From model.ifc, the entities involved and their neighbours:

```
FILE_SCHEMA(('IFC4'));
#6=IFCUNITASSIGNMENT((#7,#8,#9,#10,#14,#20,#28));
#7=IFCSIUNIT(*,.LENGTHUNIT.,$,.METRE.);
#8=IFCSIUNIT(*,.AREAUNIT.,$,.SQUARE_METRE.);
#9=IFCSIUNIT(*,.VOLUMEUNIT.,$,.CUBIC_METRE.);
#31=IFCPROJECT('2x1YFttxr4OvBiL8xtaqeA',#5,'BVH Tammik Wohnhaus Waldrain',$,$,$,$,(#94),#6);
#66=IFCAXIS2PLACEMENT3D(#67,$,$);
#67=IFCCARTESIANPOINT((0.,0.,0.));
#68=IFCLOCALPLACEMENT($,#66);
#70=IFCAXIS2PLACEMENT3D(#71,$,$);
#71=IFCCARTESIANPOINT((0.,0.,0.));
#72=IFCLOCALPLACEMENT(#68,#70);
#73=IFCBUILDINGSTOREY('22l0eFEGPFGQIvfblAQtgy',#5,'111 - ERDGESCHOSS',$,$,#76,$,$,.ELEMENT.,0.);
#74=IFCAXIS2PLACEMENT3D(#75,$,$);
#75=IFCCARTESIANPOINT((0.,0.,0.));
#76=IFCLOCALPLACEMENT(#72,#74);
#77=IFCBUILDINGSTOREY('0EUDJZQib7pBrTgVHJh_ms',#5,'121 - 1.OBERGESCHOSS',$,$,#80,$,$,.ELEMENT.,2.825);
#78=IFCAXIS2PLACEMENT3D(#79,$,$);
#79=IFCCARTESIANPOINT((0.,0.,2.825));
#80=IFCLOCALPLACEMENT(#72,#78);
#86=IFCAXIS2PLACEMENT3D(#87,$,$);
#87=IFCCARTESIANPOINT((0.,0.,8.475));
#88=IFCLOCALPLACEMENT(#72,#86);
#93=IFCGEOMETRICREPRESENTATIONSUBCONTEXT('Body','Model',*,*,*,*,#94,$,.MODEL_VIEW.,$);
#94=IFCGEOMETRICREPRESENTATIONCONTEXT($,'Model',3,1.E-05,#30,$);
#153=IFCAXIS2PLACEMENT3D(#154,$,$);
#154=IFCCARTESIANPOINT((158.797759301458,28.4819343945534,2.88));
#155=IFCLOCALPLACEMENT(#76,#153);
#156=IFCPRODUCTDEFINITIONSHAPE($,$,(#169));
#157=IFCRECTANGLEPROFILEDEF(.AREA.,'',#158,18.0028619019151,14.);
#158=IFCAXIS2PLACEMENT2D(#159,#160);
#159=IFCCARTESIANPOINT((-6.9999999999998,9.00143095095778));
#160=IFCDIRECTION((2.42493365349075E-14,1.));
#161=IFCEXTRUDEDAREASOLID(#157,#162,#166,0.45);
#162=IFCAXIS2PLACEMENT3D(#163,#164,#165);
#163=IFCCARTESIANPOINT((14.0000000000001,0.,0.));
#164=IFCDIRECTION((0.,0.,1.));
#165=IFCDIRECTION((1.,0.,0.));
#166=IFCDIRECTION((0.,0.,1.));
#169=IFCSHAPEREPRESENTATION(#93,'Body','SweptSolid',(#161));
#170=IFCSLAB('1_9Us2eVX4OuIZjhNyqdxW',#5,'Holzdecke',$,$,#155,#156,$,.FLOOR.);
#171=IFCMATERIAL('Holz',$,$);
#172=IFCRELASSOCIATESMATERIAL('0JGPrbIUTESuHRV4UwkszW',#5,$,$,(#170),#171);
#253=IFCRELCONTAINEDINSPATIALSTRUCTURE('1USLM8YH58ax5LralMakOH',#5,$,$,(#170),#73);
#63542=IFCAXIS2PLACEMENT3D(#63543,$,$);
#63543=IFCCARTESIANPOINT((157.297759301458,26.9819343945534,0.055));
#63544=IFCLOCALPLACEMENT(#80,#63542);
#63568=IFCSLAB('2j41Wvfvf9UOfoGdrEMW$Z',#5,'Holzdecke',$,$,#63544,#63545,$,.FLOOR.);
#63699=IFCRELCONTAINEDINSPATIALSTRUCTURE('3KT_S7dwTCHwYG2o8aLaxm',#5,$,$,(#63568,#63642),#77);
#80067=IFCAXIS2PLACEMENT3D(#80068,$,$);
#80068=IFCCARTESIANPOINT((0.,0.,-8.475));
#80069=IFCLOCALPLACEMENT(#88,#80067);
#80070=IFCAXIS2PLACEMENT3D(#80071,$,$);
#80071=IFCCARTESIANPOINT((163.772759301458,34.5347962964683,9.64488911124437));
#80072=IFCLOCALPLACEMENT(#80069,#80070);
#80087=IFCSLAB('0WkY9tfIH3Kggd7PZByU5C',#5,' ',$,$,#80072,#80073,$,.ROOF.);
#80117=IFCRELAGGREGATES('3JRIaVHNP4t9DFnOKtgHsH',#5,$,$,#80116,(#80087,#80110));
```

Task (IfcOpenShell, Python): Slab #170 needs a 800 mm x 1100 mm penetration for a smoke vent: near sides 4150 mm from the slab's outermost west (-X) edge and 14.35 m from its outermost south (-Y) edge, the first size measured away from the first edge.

```python
import numpy as np
import ifcopenshell
import ifcopenshell.api.feature
import ifcopenshell.api.geometry
import ifcopenshell.api.root
import ifcopenshell.geom
import ifcopenshell.util.placement
import ifcopenshell.util.representation
import ifcopenshell.util.shape
import ifcopenshell.util.unit

model = ifcopenshell.open("model.ifc")
unit_scale = ifcopenshell.util.unit.calculate_unit_scale(model)
settings = ifcopenshell.geom.settings()


def volume(element):
    """Net volume in cubic metres, openings subtracted."""
    shape = ifcopenshell.geom.create_shape(settings, element)
    return ifcopenshell.util.shape.get_volume(shape.geometry)


slab = model.by_id(170)
before = volume(slab)

# Extent in the slab's own axes, in metres. The edges named are its -X and -Y sides.
slab_shape = ifcopenshell.geom.create_shape(settings, slab)
vertices = ifcopenshell.util.shape.get_vertices(slab_shape.geometry)
x_min, y_min, bottom = vertices.min(axis=0)
top = vertices[:, 2].max()

opening = ifcopenshell.api.root.create_entity(model, ifc_class="IfcOpeningElement", name="Smoke vent opening", predefined_type="OPENING")
context = ifcopenshell.util.representation.get_context(model, "Model", "Body", "MODEL_VIEW")
width, depth = 0.8, 1.1
outline = [(0.0, 0.0), (width, 0.0), (width, depth), (0.0, depth), (0.0, 0.0)]
# Overshoot both faces by 50 mm so the cut is clean.
shape = ifcopenshell.api.geometry.add_slab_representation(
    model, context=context, depth=top - bottom + 0.1, polyline=outline
)
ifcopenshell.api.geometry.assign_representation(model, product=opening, representation=shape)

matrix = ifcopenshell.util.placement.get_local_placement(slab.ObjectPlacement)
matrix[:, 3] = matrix @ np.append(np.array([x_min + 4.15, y_min + 14.35, bottom - 0.05]) / unit_scale, 1.0)
ifcopenshell.api.geometry.edit_object_placement(model, product=opening, matrix=matrix, is_si=False)
ifcopenshell.api.feature.add_feature(model, feature=opening, element=slab)

after = volume(slab)

print(f"slab volume {before:.3f} -> {after:.3f} m3")

model.write("model_v2.ifc")
```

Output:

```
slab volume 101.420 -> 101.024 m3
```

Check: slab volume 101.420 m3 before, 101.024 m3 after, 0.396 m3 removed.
